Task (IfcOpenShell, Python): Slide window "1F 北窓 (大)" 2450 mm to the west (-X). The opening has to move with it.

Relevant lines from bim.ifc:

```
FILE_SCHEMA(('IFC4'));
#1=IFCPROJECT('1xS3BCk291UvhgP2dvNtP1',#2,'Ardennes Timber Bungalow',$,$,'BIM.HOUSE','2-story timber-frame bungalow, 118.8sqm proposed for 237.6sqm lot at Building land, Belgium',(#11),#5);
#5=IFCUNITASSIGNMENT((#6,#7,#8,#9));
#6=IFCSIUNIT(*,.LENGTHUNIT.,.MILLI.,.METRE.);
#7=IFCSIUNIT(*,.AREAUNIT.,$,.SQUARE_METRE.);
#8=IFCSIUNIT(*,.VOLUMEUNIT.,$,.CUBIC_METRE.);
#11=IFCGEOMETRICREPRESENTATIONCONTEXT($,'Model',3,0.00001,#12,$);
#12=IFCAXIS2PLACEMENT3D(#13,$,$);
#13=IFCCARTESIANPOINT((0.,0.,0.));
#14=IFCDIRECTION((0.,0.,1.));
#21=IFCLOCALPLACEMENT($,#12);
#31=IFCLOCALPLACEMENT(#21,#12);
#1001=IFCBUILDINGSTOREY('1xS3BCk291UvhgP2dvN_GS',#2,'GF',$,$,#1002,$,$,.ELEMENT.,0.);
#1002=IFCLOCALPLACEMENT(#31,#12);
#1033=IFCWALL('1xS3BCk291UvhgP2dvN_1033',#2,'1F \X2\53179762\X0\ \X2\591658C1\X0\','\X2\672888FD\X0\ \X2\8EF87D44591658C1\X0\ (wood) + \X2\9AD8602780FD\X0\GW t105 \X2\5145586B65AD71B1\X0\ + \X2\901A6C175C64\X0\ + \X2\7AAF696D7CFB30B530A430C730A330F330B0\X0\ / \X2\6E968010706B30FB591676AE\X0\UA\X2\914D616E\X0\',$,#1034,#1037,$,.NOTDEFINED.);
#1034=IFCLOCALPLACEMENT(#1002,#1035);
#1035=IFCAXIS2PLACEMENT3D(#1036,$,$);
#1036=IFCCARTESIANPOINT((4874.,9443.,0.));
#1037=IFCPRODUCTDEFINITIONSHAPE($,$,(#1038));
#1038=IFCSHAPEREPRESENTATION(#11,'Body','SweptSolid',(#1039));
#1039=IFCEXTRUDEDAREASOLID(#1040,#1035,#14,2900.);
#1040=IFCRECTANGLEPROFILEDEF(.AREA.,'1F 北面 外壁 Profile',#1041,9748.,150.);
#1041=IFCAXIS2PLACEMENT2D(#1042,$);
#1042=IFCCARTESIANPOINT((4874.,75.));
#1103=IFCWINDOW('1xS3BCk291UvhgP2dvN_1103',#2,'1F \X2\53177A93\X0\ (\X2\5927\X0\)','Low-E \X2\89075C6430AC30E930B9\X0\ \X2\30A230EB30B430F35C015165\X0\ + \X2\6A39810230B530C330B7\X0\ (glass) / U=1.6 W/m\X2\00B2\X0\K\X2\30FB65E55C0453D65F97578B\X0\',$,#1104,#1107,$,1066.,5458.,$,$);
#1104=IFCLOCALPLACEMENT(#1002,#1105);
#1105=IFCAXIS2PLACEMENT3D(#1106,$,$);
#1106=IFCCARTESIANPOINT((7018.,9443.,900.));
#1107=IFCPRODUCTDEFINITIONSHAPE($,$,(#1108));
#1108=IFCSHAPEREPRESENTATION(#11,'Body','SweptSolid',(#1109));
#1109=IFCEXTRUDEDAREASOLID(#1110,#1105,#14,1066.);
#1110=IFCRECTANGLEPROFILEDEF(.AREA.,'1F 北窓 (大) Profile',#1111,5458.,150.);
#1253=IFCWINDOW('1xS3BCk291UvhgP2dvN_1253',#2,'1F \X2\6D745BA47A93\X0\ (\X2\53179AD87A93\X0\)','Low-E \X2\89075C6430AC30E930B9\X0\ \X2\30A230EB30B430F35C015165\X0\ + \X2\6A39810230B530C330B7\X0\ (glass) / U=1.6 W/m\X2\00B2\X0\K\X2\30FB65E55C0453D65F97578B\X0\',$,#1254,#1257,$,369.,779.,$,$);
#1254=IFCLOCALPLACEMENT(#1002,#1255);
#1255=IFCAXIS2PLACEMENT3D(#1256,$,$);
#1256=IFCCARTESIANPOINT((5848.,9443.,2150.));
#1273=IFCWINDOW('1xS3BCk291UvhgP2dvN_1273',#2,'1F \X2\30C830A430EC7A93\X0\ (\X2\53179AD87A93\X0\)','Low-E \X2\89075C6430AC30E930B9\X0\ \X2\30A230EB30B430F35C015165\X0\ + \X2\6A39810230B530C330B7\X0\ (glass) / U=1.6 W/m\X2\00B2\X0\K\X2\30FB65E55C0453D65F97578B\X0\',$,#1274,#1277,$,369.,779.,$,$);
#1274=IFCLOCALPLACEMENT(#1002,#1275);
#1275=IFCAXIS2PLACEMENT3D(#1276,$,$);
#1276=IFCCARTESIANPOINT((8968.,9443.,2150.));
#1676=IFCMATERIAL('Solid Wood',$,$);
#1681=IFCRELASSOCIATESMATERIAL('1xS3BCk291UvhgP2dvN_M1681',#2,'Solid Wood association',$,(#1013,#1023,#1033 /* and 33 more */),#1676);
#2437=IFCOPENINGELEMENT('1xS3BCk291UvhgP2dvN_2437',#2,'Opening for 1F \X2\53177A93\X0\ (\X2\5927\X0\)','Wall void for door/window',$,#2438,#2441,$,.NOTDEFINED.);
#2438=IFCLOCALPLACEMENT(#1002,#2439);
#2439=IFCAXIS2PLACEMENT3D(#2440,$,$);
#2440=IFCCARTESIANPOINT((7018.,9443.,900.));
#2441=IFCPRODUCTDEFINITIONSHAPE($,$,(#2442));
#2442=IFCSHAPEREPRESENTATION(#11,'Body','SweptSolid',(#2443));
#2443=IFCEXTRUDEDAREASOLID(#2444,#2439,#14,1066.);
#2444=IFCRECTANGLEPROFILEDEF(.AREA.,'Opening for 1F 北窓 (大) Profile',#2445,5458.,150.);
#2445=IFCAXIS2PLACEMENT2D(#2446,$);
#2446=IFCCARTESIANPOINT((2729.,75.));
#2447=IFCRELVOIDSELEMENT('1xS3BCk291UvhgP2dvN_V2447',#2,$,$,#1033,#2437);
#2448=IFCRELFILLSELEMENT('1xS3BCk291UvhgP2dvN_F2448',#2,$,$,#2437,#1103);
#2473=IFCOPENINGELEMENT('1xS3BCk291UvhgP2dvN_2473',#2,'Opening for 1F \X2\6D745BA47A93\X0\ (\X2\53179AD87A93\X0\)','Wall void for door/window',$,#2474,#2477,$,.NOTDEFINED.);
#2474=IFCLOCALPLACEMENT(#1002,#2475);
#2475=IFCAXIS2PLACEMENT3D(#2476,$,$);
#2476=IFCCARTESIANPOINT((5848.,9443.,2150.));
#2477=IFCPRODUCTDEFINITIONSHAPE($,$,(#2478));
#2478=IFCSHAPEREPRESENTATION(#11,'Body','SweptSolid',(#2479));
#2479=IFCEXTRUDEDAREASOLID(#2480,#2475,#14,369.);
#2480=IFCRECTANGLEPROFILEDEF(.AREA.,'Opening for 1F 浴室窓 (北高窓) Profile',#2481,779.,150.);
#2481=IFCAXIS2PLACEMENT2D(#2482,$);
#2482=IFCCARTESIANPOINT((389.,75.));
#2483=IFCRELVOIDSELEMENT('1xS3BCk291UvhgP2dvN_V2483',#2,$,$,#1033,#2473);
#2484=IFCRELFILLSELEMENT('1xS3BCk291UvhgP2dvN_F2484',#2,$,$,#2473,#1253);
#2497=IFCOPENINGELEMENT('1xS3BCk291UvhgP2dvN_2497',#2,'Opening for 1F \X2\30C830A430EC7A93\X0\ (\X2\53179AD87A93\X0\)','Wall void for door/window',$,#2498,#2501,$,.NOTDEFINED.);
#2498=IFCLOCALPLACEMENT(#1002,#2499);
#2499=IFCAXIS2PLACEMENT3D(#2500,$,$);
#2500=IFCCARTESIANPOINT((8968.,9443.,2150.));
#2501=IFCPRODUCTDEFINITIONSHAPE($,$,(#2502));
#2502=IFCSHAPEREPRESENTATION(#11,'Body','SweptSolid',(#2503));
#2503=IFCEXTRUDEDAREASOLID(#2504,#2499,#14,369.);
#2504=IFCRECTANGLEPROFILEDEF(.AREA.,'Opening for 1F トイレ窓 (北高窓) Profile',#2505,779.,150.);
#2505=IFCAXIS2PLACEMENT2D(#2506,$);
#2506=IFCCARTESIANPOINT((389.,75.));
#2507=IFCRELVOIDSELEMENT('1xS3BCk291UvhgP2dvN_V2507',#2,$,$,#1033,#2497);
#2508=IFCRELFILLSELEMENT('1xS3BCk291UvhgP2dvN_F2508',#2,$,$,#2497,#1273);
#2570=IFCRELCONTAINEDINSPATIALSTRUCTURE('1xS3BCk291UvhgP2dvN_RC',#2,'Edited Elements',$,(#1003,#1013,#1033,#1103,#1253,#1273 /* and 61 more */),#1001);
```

```python
import ifcopenshell
import ifcopenshell.api.geometry
import ifcopenshell.util.placement

model = ifcopenshell.open("bim.ifc")

window = model.by_guid("1xS3BCk291UvhgP2dvN_1103")
opening = window.FillsVoids[0].RelatingOpeningElement
wall = opening.VoidsElements[0].RelatingBuildingElement

wall_matrix = ifcopenshell.util.placement.get_local_placement(wall.ObjectPlacement)
shift = wall_matrix[:3, 0] * -2450.0
before = ifcopenshell.util.placement.get_local_placement(window.ObjectPlacement)[:3, 3].copy()

# The window is not placed relative to its opening, so move both.
for product in (opening, window):
    matrix = ifcopenshell.util.placement.get_local_placement(product.ObjectPlacement)
    matrix[:3, 3] += shift
    ifcopenshell.api.geometry.edit_object_placement(model, product=product, matrix=matrix, is_si=False)

after = ifcopenshell.util.placement.get_local_placement(window.ObjectPlacement)[:3, 3]
print("window moved by", (after - before).round(3) + 0.0)

model.write("bim_updated.ifc")
```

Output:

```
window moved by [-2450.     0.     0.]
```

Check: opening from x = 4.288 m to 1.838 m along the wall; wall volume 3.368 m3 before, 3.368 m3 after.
